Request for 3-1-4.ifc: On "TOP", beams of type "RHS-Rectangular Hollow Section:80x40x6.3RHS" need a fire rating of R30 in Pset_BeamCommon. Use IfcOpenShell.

First a look at what the model holds.

```python
import ifcopenshell
import ifcopenshell.util.element

model = ifcopenshell.open("3-1-4.ifc")
print(model.schema)
storey = next(s for s in model.by_type("IfcBuildingStorey") if s.Name == "TOP")
beams = [e for e in ifcopenshell.util.element.get_decomposition(storey) if e.is_a("IfcBeam")]
seen = {}
for e in beams:
    element_type = ifcopenshell.util.element.get_type(e)
    key = (element_type.Name if element_type != e and element_type else None, ifcopenshell.util.element.get_pset(e, "Pset_BeamCommon", "FireRating"))
    seen[key] = seen.get(key, 0) + 1
for (name, value), count in sorted(seen.items(), key=str):
    print(count, "x", name, "|", value)
```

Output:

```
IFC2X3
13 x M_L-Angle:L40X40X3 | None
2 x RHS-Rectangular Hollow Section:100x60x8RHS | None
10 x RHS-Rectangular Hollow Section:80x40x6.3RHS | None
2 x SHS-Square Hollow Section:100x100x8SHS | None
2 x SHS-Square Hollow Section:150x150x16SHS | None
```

```python
import ifcopenshell
import ifcopenshell.api.pset
import ifcopenshell.util.element

model = ifcopenshell.open("3-1-4.ifc")

storey = next(s for s in model.by_type("IfcBuildingStorey") if s.Name == "TOP")
beams = [e for e in ifcopenshell.util.element.get_decomposition(storey) if e.is_a("IfcBeam")]

count = 0
for e in beams:
    element_type = ifcopenshell.util.element.get_type(e)
    if element_type in (None, e) or element_type.Name != "RHS-Rectangular Hollow Section:80x40x6.3RHS":
        continue
    # add_pset returns the element's existing set when there is one.
    pset = ifcopenshell.api.pset.add_pset(model, product=e, name="Pset_BeamCommon")
    ifcopenshell.api.pset.edit_pset(model, pset=pset, properties={"FireRating": "R30"})
    count += 1

print(count, "beams updated")

model.write("3-1-4_updated.ifc")
```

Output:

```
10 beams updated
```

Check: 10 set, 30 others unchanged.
